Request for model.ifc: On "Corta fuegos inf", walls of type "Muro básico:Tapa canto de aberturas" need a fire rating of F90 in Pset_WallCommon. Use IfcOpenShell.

First a look at what the model holds.

```python
import ifcopenshell
import ifcopenshell.util.element

model = ifcopenshell.open("model.ifc")
print(model.schema)
storey = next(s for s in model.by_type("IfcBuildingStorey") if s.Name == "Corta fuegos inf")
walls = [e for e in ifcopenshell.util.element.get_decomposition(storey) if e.is_a("IfcWall")]
seen = {}
for e in walls:
    element_type = ifcopenshell.util.element.get_type(e)
    key = (element_type.Name if element_type != e and element_type else None, ifcopenshell.util.element.get_pset(e, "Pset_WallCommon", "FireRating"))
    seen[key] = seen.get(key, 0) + 1
for (name, value), count in sorted(seen.items(), key=str):
    print(count, "x", name, "|", value)
```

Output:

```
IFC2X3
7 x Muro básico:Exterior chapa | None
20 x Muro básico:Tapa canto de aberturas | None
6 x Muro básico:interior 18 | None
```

```python
import ifcopenshell
import ifcopenshell.api.pset
import ifcopenshell.util.element

model = ifcopenshell.open("model.ifc")

storey = next(s for s in model.by_type("IfcBuildingStorey") if s.Name == "Corta fuegos inf")
walls = [e for e in ifcopenshell.util.element.get_decomposition(storey) if e.is_a("IfcWall")]

count = 0
for e in walls:
    element_type = ifcopenshell.util.element.get_type(e)
    if element_type in (None, e) or element_type.Name != "Muro básico:Tapa canto de aberturas":
        continue
    # add_pset returns the element's existing set when there is one.
    pset = ifcopenshell.api.pset.add_pset(model, product=e, name="Pset_WallCommon")
    ifcopenshell.api.pset.edit_pset(model, pset=pset, properties={"FireRating": "F90"})
    count += 1

print(count, "walls updated")

model.write("model_edited.ifc")
```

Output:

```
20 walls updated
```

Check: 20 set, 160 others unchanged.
